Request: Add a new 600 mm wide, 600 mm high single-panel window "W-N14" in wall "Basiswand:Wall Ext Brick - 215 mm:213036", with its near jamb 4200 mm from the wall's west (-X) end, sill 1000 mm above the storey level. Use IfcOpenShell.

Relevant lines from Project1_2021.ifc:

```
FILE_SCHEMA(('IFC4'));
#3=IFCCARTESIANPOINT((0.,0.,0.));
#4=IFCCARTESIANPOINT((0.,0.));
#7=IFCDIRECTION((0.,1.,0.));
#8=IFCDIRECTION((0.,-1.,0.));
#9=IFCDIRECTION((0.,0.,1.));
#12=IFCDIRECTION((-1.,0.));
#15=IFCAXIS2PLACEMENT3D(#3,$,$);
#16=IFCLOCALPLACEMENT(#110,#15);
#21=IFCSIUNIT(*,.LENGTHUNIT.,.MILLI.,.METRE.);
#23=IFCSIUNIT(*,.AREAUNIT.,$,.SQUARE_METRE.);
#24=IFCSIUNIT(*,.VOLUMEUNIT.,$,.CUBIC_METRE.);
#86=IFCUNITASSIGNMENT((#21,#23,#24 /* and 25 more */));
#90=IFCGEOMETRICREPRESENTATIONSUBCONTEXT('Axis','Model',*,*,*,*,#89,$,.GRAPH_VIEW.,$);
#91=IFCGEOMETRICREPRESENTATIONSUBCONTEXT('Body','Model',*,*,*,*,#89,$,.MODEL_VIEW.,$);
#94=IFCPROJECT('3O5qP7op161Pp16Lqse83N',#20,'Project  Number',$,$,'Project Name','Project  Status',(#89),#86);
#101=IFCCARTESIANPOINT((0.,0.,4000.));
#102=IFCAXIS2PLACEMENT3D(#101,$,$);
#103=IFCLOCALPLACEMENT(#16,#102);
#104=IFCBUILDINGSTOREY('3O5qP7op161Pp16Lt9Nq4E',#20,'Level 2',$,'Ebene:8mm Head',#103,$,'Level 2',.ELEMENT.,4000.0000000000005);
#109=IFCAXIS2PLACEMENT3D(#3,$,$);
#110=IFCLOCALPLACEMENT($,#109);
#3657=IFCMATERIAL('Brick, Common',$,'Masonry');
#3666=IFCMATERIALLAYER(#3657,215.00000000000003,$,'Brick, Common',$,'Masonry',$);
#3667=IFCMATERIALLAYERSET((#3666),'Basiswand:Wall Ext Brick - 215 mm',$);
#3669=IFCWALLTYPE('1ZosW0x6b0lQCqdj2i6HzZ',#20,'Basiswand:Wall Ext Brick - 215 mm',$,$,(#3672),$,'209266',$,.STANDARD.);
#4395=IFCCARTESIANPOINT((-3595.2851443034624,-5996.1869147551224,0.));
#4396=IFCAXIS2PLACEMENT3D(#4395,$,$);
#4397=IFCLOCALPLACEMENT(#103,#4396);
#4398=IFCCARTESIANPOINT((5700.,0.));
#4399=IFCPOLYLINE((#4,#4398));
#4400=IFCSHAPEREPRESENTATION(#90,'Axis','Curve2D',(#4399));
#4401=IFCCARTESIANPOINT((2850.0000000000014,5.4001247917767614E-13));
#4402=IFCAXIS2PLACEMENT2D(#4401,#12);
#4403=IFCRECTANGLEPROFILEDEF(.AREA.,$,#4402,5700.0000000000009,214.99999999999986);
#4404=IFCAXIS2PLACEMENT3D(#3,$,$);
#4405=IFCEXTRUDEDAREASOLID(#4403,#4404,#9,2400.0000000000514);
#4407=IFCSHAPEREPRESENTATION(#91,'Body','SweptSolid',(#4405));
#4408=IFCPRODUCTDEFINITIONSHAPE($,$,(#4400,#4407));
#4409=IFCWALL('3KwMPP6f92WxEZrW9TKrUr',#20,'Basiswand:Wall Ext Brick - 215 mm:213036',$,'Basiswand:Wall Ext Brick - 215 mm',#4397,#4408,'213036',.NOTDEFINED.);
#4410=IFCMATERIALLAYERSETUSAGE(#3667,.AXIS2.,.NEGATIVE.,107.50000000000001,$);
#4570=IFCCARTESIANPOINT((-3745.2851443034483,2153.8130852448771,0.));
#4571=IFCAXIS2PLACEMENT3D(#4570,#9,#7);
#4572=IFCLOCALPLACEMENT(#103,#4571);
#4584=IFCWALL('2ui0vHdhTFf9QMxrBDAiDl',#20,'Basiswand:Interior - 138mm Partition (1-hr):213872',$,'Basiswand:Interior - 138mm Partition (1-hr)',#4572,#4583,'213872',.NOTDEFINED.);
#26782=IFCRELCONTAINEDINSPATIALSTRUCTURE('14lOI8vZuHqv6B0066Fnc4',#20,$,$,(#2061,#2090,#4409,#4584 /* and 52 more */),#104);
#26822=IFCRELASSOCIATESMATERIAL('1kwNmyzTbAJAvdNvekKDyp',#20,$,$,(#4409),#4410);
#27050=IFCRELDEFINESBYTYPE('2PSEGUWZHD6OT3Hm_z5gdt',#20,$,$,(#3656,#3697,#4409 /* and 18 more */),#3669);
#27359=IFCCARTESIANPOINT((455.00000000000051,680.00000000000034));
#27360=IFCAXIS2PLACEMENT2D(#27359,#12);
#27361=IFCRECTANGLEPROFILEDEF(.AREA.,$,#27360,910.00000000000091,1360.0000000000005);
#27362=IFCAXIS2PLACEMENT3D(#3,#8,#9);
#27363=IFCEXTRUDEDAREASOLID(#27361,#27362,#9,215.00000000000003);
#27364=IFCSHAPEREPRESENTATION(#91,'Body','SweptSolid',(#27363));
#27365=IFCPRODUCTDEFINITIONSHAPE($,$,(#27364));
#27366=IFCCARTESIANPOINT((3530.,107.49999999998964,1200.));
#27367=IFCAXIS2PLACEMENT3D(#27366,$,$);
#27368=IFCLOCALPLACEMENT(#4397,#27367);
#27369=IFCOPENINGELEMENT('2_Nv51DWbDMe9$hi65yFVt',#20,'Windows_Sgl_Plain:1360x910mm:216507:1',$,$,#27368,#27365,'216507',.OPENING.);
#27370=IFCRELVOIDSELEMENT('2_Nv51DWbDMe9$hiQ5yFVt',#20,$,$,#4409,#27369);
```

```python
import numpy as np
import ifcopenshell
import ifcopenshell.api.feature
import ifcopenshell.api.geometry
import ifcopenshell.api.root
import ifcopenshell.api.spatial
import ifcopenshell.geom
import ifcopenshell.util.element
import ifcopenshell.util.placement
import ifcopenshell.util.representation
import ifcopenshell.util.shape
import ifcopenshell.util.unit

model = ifcopenshell.open("Project1_2021.ifc")
unit_scale = ifcopenshell.util.unit.calculate_unit_scale(model)
settings = ifcopenshell.geom.settings()


def volume(element):
    """Net volume in cubic metres, openings subtracted."""
    shape = ifcopenshell.geom.create_shape(settings, element)
    return ifcopenshell.util.shape.get_volume(shape.geometry)


wall = model.by_guid("3KwMPP6f92WxEZrW9TKrUr")
storey = ifcopenshell.util.element.get_container(wall, ifc_class="IfcBuildingStorey")
context = ifcopenshell.util.representation.get_context(model, "Model", "Body", "MODEL_VIEW")
before = volume(wall)

width, height, from_end, sill = 0.6, 0.6, 4.2, 1  # metres

# The wall runs along its own X axis, and the end named is its -X end.
wall_shape = ifcopenshell.geom.create_shape(settings, wall)
x, y, z = ifcopenshell.util.shape.get_vertices(wall_shape.geometry).T
start = x.min() + from_end
face, thickness = float(y.min()), float(y.max() - y.min())
wall_matrix = ifcopenshell.util.placement.get_local_placement(wall.ObjectPlacement)
level = ifcopenshell.util.placement.get_local_placement(storey.ObjectPlacement)[2, 3]


def in_wall(x, y):
    """Placement at x, y metres in the wall's axes, at sill height."""
    matrix = wall_matrix.copy()
    matrix[:, 3] = wall_matrix @ np.array([x / unit_scale, y / unit_scale, 0.0, 1.0])
    matrix[2, 3] = level + sill / unit_scale
    return matrix


# Opening: a box that overshoots both wall faces by 50 mm.
opening = ifcopenshell.api.root.create_entity(model, ifc_class="IfcOpeningElement", predefined_type="OPENING")
box = ifcopenshell.api.geometry.add_wall_representation(
    model, context=context, length=width, height=height, thickness=thickness + 0.1
)
ifcopenshell.api.geometry.assign_representation(model, product=opening, representation=box)
ifcopenshell.api.geometry.edit_object_placement(model, product=opening, matrix=in_wall(start, face - 0.05), is_si=False)
ifcopenshell.api.feature.add_feature(model, feature=opening, element=wall)

window = ifcopenshell.api.root.create_entity(model, ifc_class="IfcWindow", name="W-N14", predefined_type="WINDOW")
window.OverallWidth, window.OverallHeight = width / unit_scale, height / unit_scale
window.PartitioningType = "SINGLE_PANEL"
body = ifcopenshell.api.geometry.add_window_representation(
    model,
    context=context,
    overall_width=window.OverallWidth,
    overall_height=window.OverallHeight,
    partition_type="SINGLE_PANEL",
)
ifcopenshell.api.geometry.assign_representation(model, product=window, representation=body)
ifcopenshell.api.spatial.assign_container(model, products=[window], relating_structure=storey)
ifcopenshell.api.feature.add_filling(model, opening=opening, element=window)

# Centre the window in the wall's thickness.
ifcopenshell.api.geometry.edit_object_placement(model, product=window, matrix=in_wall(start, face), is_si=False)
window_shape = ifcopenshell.geom.create_shape(settings, window)
depth = ifcopenshell.util.shape.get_vertices(window_shape.geometry)[:, 1]
offset = face + thickness / 2 - (depth.min() + depth.max()) / 2
ifcopenshell.api.geometry.edit_object_placement(model, product=window, matrix=in_wall(start, offset), is_si=False)

after = volume(wall)

print(f"wall volume {before:.3f} -> {after:.3f} m3")

model.write("Project1_2021_updated.ifc")
```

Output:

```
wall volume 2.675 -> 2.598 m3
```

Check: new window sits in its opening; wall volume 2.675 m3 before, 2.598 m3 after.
